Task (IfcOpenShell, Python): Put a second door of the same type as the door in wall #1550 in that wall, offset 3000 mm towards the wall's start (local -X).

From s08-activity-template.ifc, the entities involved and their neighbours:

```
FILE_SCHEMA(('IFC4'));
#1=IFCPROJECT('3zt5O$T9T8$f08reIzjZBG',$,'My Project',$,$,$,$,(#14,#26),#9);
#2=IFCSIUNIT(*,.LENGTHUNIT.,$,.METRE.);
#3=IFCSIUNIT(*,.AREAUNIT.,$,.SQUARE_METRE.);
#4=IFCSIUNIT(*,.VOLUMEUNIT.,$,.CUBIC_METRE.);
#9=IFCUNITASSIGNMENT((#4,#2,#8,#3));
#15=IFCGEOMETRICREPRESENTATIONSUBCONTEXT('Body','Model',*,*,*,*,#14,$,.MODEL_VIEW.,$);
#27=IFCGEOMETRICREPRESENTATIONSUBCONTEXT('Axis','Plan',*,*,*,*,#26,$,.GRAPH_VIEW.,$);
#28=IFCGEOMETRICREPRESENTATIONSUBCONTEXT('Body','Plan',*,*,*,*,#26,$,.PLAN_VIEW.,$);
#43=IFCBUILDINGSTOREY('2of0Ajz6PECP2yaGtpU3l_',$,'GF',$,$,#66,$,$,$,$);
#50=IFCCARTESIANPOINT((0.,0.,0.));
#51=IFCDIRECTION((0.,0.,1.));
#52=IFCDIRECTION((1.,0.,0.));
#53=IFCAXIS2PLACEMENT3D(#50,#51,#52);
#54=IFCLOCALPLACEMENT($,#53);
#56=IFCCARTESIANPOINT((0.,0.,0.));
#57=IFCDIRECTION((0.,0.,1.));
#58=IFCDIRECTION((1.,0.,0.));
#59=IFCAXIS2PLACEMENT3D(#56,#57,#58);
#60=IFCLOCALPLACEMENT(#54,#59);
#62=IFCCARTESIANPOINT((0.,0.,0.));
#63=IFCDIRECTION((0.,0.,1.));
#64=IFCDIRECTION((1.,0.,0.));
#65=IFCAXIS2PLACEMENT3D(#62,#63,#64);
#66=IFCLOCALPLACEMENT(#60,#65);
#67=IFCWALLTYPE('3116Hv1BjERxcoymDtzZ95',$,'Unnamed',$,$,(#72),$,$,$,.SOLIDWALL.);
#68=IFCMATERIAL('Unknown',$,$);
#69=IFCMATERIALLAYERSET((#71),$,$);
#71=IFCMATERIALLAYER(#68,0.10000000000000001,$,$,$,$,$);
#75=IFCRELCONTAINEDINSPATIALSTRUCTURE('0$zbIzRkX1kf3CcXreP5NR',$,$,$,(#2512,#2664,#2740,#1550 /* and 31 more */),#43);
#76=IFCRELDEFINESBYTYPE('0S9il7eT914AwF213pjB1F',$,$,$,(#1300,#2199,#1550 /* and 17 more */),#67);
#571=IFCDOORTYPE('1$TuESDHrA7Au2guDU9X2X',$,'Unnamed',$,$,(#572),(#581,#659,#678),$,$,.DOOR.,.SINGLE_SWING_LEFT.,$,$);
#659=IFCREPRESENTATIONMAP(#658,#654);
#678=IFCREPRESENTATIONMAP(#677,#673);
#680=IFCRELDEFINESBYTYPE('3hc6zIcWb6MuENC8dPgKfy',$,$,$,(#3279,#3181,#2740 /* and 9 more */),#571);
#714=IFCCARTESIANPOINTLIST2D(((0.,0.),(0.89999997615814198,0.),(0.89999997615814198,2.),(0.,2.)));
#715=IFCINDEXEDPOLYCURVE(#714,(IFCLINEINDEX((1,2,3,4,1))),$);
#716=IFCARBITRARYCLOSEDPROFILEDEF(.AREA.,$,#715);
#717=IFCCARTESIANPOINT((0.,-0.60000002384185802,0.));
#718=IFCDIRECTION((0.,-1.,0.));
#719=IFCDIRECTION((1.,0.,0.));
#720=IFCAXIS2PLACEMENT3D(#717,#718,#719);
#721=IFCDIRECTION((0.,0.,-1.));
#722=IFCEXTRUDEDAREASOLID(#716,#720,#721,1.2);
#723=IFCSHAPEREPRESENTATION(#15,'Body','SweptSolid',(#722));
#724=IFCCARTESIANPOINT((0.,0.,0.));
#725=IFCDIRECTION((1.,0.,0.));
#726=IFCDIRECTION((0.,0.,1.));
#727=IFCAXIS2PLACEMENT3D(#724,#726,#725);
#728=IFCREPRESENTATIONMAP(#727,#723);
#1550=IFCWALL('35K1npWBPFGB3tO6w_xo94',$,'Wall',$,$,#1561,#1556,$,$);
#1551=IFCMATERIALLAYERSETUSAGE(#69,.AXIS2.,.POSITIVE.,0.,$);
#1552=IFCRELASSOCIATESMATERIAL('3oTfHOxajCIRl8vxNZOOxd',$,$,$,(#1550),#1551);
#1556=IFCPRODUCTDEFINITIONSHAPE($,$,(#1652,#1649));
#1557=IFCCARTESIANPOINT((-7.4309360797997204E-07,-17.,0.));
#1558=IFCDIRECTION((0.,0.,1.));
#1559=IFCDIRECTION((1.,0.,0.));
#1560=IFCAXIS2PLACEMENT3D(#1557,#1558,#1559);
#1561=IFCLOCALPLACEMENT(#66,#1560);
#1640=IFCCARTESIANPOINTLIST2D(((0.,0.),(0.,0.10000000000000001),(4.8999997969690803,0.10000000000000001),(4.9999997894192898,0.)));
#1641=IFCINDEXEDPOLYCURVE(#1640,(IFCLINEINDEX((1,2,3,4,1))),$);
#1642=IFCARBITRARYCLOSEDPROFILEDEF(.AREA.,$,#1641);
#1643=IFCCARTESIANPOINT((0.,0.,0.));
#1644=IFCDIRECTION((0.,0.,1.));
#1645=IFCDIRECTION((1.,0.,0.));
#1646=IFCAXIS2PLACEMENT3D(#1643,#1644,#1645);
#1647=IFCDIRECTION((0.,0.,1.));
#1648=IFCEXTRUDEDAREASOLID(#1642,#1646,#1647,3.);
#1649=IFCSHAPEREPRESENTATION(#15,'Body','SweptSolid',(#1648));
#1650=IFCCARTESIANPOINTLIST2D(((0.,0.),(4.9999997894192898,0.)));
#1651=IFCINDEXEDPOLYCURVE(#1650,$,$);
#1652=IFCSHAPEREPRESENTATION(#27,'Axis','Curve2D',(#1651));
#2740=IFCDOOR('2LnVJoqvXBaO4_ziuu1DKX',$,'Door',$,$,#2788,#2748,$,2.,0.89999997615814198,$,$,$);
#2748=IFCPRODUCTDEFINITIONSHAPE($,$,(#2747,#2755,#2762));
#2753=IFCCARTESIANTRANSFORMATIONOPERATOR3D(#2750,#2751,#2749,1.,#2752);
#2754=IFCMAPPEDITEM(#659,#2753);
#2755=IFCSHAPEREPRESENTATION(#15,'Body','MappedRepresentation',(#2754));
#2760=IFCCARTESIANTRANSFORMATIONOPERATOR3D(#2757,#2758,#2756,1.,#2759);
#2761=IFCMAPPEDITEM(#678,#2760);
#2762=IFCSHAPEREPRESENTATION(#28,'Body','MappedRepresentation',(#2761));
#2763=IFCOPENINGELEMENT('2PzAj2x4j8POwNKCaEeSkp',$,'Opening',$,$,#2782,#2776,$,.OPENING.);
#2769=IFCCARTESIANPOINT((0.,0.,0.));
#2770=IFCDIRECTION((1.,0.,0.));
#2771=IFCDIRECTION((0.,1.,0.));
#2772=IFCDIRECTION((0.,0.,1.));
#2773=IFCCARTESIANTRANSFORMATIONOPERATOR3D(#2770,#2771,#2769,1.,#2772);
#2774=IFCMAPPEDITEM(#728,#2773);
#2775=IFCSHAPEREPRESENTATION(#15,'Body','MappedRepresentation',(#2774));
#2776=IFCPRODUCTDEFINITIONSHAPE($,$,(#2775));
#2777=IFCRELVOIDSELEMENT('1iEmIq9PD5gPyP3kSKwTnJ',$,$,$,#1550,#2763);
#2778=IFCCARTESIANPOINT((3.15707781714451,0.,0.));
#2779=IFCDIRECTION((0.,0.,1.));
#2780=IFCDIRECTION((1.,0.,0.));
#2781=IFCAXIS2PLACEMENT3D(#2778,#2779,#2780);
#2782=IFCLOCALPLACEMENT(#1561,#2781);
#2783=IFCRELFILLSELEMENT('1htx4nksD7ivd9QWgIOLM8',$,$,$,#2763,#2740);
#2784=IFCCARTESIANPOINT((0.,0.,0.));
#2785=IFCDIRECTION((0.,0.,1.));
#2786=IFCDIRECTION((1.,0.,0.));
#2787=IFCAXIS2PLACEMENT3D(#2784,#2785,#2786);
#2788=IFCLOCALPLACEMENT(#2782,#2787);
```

```python
import ifcopenshell
import ifcopenshell.api.feature
import ifcopenshell.api.geometry
import ifcopenshell.api.root
import ifcopenshell.geom
import ifcopenshell.util.element
import ifcopenshell.util.placement
import ifcopenshell.util.shape
import ifcopenshell.util.unit

model = ifcopenshell.open("s08-activity-template.ifc")
unit_scale = ifcopenshell.util.unit.calculate_unit_scale(model)
settings = ifcopenshell.geom.settings()


def volume(element):
    """Net volume in cubic metres, openings subtracted."""
    shape = ifcopenshell.geom.create_shape(settings, element)
    return ifcopenshell.util.shape.get_volume(shape.geometry)


door = model.by_id(2740)
opening = door.FillsVoids[0].RelatingOpeningElement
wall = opening.VoidsElements[0].RelatingBuildingElement
before = volume(wall)
shift = ifcopenshell.util.placement.get_local_placement(wall.ObjectPlacement)[:3, 0] * -3 / unit_scale

# copy_class copies the void relationship, type, container and properties, but no geometry.
new_opening = ifcopenshell.api.root.copy_class(model, product=opening)
new_opening.Representation = ifcopenshell.util.element.copy_deep(
    model, opening.Representation, exclude=["IfcGeometricRepresentationContext", "IfcRepresentationMap"]
)
new_door = ifcopenshell.api.root.copy_class(model, product=door)
new_door.Representation = ifcopenshell.util.element.copy_deep(
    model, door.Representation, exclude=["IfcGeometricRepresentationContext", "IfcRepresentationMap"]
)
ifcopenshell.api.feature.add_filling(model, opening=new_opening, element=new_door)

for old, new in ((opening, new_opening), (door, new_door)):
    matrix = ifcopenshell.util.placement.get_local_placement(old.ObjectPlacement)
    matrix[:3, 3] += shift
    ifcopenshell.api.geometry.edit_object_placement(model, product=new, matrix=matrix, is_si=False)

after = volume(wall)

print(f"wall volume {before:.3f} -> {after:.3f} m3")

model.write("s08-activity-template_edited.ifc")
```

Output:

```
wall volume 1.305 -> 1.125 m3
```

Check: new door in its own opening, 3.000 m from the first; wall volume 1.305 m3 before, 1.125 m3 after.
